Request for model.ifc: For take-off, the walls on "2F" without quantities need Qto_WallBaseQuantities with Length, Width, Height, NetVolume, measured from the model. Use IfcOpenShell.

First a look at what the model holds.

```python
import ifcopenshell
import ifcopenshell.util.element
import ifcopenshell.util.unit

model = ifcopenshell.open("model.ifc")
print(model.schema)
for unit_type in ("LENGTHUNIT", "AREAUNIT", "VOLUMEUNIT"):
    print(unit_type, ifcopenshell.util.unit.calculate_unit_scale(model, unit_type))
storey = next(s for s in model.by_type("IfcBuildingStorey") if s.Name == "2F")
walls = [e for e in ifcopenshell.util.element.get_decomposition(storey) if e.is_a("IfcWall")]
for e in sorted(walls, key=lambda e: e.id()):
    print(e.id(), e.is_a(), e.Name, list(ifcopenshell.util.element.get_psets(e, qtos_only=True)), sep=" | ")
```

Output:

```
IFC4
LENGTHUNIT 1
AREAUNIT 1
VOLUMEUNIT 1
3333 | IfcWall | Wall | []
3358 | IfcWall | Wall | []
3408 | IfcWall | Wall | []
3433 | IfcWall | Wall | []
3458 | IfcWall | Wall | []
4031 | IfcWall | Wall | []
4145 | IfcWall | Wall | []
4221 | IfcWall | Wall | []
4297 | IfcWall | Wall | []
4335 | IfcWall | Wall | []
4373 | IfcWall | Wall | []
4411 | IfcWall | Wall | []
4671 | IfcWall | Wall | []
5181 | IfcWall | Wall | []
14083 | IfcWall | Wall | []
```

```python
import ifcopenshell
import ifcopenshell.api.pset
import ifcopenshell.geom
import ifcopenshell.util.element
import ifcopenshell.util.shape
import ifcopenshell.util.unit

model = ifcopenshell.open("model.ifc")
unit_scale = ifcopenshell.util.unit.calculate_unit_scale(model)
volume_scale = ifcopenshell.util.unit.calculate_unit_scale(model, "VOLUMEUNIT")
settings = ifcopenshell.geom.settings()

storey = next(s for s in model.by_type("IfcBuildingStorey") if s.Name == "2F")
walls = [e for e in ifcopenshell.util.element.get_decomposition(storey) if e.is_a("IfcWall")]

for e in sorted(walls, key=lambda e: e.id()):
    if ifcopenshell.util.element.get_psets(e, qtos_only=True, should_inherit=False):
        continue
    # Geometry comes back in metres, in the element's own axes.
    shape = ifcopenshell.geom.create_shape(settings, e)
    values = {
        "Length": ifcopenshell.util.shape.get_x(shape.geometry) / unit_scale,
        "Width": ifcopenshell.util.shape.get_y(shape.geometry) / unit_scale,
        "Height": ifcopenshell.util.shape.get_z(shape.geometry) / unit_scale,
        "NetVolume": ifcopenshell.util.shape.get_volume(shape.geometry) / volume_scale,
    }
    qto = ifcopenshell.api.pset.add_qto(model, product=e, name="Qto_WallBaseQuantities")
    ifcopenshell.api.pset.edit_qto(model, qto=qto, properties=values)
    print(e.id(), {k: round(v, 3) for k, v in values.items()})

model.write("model_rev.ifc")
```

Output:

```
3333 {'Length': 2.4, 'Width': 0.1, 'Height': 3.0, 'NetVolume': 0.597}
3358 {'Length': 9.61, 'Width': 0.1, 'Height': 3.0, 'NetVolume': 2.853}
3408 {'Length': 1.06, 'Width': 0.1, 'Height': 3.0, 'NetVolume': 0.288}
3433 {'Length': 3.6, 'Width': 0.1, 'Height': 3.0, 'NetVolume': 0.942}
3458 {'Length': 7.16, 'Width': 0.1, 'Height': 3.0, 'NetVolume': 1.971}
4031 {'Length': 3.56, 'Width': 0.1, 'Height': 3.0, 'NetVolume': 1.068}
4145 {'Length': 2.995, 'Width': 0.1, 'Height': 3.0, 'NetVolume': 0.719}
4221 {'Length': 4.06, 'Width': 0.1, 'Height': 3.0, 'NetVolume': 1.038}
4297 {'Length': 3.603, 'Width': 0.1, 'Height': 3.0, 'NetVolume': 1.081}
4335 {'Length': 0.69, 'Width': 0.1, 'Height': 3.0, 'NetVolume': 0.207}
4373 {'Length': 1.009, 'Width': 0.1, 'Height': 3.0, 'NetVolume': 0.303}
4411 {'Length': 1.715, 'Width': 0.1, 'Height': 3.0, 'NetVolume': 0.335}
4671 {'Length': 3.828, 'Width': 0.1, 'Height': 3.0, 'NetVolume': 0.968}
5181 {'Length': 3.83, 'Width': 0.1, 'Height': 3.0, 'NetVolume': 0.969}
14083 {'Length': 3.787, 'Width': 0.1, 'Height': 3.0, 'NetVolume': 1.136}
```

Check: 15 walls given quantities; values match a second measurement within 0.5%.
